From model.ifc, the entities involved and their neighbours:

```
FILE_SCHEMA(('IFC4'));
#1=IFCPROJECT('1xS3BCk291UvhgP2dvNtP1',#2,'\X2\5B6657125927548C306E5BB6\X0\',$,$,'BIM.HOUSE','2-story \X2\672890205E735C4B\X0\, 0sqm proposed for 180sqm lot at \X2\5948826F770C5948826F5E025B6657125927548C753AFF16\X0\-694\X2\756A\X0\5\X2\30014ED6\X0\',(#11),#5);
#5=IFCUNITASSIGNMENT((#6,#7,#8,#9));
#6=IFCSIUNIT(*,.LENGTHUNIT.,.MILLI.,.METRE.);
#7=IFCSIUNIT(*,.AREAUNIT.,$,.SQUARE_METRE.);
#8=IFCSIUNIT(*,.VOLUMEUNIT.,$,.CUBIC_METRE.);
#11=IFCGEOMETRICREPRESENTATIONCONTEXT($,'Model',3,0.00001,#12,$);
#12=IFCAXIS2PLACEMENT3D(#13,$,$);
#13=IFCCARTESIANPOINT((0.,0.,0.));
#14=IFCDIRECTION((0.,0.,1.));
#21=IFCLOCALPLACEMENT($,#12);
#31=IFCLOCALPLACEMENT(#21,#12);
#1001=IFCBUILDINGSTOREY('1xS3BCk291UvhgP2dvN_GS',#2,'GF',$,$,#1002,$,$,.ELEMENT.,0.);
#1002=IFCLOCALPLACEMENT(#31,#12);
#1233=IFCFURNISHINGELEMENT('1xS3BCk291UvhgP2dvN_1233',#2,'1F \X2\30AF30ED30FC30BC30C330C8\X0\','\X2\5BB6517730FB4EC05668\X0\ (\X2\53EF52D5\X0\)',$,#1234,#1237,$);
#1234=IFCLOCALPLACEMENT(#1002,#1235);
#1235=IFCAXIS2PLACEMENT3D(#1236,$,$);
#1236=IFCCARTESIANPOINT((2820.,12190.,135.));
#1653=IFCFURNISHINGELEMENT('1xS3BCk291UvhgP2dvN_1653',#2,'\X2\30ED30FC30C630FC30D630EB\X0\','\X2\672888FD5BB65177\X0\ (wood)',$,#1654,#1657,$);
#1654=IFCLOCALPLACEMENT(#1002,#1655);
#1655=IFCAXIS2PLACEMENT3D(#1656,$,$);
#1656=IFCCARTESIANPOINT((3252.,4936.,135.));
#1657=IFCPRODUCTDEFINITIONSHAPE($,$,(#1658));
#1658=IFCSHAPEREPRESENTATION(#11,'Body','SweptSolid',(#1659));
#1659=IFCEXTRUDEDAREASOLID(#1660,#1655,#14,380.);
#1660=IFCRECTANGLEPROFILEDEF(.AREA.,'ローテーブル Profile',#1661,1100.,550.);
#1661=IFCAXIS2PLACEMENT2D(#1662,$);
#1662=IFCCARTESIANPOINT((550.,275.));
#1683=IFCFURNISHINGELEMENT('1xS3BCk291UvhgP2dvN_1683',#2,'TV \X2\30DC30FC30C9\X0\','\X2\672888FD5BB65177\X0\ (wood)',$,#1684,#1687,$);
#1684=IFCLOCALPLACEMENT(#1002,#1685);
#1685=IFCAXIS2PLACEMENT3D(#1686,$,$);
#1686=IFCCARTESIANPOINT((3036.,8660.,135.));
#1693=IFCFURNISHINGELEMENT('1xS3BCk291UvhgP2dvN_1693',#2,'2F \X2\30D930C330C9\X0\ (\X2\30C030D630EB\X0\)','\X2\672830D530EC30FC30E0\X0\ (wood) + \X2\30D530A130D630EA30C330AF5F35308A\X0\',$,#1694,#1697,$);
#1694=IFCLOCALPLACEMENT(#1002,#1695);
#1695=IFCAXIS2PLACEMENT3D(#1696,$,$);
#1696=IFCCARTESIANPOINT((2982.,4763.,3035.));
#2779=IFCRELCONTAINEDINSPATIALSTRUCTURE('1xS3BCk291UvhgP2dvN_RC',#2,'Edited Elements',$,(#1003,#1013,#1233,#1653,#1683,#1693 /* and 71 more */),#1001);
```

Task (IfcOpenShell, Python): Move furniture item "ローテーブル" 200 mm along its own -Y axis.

```python
import ifcopenshell
import ifcopenshell.api.geometry
import ifcopenshell.util.placement

model = ifcopenshell.open("model.ifc")

item = model.by_id(1653)
matrix = ifcopenshell.util.placement.get_local_placement(item.ObjectPlacement)
matrix[:3, 3] -= matrix[:3, 1] * 200.0
ifcopenshell.api.geometry.edit_object_placement(model, product=item, matrix=matrix, is_si=False)

print(ifcopenshell.util.placement.get_local_placement(item.ObjectPlacement).round(3) + 0.0)

model.write("model_edited.ifc")
```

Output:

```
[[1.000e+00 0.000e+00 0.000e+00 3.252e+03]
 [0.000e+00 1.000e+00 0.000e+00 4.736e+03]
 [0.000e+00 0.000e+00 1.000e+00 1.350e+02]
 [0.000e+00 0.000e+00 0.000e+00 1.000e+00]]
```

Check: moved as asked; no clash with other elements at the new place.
